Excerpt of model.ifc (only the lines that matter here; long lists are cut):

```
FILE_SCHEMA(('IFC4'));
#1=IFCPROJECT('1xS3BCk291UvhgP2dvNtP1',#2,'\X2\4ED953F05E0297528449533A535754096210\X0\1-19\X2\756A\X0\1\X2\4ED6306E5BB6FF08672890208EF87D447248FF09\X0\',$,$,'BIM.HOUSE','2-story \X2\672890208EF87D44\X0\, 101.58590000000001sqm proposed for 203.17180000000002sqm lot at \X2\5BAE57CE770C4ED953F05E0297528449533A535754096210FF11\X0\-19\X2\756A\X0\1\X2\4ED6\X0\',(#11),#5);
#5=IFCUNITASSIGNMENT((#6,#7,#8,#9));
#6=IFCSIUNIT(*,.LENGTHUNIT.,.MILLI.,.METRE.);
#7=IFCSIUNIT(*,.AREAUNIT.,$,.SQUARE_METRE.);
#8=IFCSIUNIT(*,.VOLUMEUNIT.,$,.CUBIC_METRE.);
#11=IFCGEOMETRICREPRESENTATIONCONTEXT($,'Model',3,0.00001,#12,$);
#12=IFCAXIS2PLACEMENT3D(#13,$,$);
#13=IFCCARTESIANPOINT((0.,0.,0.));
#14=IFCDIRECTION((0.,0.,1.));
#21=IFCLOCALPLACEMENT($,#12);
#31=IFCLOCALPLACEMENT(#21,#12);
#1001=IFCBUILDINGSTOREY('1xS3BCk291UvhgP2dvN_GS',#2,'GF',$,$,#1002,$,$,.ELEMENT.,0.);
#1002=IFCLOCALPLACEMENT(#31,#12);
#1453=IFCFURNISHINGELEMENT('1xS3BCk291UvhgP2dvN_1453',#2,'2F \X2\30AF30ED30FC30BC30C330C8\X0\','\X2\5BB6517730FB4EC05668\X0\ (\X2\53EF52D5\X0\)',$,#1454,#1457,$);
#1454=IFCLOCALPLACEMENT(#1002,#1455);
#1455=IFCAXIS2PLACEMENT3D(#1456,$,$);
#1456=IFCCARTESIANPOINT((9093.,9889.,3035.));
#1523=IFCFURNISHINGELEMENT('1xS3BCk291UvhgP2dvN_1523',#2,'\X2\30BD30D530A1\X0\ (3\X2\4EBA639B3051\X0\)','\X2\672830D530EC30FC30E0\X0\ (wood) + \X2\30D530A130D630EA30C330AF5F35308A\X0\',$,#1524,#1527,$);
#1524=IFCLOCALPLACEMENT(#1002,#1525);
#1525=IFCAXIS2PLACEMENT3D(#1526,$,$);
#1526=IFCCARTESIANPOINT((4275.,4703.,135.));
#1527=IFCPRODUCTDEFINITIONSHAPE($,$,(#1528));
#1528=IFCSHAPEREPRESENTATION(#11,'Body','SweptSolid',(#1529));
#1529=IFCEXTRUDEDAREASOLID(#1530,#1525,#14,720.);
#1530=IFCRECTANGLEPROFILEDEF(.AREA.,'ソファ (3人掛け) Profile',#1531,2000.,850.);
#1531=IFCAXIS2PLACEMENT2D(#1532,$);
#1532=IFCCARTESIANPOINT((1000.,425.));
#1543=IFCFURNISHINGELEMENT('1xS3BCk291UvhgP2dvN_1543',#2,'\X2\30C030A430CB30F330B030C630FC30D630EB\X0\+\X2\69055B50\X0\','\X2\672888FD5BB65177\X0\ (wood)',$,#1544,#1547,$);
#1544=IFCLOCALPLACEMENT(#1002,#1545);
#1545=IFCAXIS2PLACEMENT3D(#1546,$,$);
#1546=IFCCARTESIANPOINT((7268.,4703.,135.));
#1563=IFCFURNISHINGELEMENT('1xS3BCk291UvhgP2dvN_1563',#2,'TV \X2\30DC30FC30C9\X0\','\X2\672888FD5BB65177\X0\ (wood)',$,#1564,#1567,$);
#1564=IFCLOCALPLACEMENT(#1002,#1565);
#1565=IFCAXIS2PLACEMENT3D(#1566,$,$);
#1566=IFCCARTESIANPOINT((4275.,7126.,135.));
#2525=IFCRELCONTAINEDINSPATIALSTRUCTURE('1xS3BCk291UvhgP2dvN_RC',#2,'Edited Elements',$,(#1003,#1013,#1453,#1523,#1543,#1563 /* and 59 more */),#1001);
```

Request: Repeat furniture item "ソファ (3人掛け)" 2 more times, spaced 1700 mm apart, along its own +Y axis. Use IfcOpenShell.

```python
import ifcopenshell
import ifcopenshell.api.geometry
import ifcopenshell.api.root
import ifcopenshell.util.element
import ifcopenshell.util.placement
import ifcopenshell.util.unit

model = ifcopenshell.open("model.ifc")
unit_scale = ifcopenshell.util.unit.calculate_unit_scale(model)


def reuse_history(source, copy):
    """copy_class also copies each property set's owner history, people and application; keep the originals."""
    for rel in copy.IsDefinedBy:
        if rel.is_a("IfcRelDefinesByProperties") and (history := rel.RelatingPropertyDefinition.OwnerHistory):
            rel.RelatingPropertyDefinition.OwnerHistory = source.OwnerHistory
            ifcopenshell.util.element.remove_deep2(model, history)


source = model.by_guid("1xS3BCk291UvhgP2dvN_1523")
base = ifcopenshell.util.placement.get_local_placement(source.ObjectPlacement)
step = base[:3, 1] * 1.7 / unit_scale

for i in range(1, 3):
    copy = ifcopenshell.api.root.copy_class(model, product=source)
    copy.Representation = ifcopenshell.util.element.copy_deep(
        model, source.Representation, exclude=["IfcGeometricRepresentationContext", "IfcRepresentationMap"]
    )
    reuse_history(source, copy)
    matrix = base.copy()
    matrix[:3, 3] += i * step
    print("added at", matrix[:3, 3].round(3) + 0.0)
    ifcopenshell.api.geometry.edit_object_placement(model, product=copy, matrix=matrix, is_si=False)

model.write("model_edited.ifc")
```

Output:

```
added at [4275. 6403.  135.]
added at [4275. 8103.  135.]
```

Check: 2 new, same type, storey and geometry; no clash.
